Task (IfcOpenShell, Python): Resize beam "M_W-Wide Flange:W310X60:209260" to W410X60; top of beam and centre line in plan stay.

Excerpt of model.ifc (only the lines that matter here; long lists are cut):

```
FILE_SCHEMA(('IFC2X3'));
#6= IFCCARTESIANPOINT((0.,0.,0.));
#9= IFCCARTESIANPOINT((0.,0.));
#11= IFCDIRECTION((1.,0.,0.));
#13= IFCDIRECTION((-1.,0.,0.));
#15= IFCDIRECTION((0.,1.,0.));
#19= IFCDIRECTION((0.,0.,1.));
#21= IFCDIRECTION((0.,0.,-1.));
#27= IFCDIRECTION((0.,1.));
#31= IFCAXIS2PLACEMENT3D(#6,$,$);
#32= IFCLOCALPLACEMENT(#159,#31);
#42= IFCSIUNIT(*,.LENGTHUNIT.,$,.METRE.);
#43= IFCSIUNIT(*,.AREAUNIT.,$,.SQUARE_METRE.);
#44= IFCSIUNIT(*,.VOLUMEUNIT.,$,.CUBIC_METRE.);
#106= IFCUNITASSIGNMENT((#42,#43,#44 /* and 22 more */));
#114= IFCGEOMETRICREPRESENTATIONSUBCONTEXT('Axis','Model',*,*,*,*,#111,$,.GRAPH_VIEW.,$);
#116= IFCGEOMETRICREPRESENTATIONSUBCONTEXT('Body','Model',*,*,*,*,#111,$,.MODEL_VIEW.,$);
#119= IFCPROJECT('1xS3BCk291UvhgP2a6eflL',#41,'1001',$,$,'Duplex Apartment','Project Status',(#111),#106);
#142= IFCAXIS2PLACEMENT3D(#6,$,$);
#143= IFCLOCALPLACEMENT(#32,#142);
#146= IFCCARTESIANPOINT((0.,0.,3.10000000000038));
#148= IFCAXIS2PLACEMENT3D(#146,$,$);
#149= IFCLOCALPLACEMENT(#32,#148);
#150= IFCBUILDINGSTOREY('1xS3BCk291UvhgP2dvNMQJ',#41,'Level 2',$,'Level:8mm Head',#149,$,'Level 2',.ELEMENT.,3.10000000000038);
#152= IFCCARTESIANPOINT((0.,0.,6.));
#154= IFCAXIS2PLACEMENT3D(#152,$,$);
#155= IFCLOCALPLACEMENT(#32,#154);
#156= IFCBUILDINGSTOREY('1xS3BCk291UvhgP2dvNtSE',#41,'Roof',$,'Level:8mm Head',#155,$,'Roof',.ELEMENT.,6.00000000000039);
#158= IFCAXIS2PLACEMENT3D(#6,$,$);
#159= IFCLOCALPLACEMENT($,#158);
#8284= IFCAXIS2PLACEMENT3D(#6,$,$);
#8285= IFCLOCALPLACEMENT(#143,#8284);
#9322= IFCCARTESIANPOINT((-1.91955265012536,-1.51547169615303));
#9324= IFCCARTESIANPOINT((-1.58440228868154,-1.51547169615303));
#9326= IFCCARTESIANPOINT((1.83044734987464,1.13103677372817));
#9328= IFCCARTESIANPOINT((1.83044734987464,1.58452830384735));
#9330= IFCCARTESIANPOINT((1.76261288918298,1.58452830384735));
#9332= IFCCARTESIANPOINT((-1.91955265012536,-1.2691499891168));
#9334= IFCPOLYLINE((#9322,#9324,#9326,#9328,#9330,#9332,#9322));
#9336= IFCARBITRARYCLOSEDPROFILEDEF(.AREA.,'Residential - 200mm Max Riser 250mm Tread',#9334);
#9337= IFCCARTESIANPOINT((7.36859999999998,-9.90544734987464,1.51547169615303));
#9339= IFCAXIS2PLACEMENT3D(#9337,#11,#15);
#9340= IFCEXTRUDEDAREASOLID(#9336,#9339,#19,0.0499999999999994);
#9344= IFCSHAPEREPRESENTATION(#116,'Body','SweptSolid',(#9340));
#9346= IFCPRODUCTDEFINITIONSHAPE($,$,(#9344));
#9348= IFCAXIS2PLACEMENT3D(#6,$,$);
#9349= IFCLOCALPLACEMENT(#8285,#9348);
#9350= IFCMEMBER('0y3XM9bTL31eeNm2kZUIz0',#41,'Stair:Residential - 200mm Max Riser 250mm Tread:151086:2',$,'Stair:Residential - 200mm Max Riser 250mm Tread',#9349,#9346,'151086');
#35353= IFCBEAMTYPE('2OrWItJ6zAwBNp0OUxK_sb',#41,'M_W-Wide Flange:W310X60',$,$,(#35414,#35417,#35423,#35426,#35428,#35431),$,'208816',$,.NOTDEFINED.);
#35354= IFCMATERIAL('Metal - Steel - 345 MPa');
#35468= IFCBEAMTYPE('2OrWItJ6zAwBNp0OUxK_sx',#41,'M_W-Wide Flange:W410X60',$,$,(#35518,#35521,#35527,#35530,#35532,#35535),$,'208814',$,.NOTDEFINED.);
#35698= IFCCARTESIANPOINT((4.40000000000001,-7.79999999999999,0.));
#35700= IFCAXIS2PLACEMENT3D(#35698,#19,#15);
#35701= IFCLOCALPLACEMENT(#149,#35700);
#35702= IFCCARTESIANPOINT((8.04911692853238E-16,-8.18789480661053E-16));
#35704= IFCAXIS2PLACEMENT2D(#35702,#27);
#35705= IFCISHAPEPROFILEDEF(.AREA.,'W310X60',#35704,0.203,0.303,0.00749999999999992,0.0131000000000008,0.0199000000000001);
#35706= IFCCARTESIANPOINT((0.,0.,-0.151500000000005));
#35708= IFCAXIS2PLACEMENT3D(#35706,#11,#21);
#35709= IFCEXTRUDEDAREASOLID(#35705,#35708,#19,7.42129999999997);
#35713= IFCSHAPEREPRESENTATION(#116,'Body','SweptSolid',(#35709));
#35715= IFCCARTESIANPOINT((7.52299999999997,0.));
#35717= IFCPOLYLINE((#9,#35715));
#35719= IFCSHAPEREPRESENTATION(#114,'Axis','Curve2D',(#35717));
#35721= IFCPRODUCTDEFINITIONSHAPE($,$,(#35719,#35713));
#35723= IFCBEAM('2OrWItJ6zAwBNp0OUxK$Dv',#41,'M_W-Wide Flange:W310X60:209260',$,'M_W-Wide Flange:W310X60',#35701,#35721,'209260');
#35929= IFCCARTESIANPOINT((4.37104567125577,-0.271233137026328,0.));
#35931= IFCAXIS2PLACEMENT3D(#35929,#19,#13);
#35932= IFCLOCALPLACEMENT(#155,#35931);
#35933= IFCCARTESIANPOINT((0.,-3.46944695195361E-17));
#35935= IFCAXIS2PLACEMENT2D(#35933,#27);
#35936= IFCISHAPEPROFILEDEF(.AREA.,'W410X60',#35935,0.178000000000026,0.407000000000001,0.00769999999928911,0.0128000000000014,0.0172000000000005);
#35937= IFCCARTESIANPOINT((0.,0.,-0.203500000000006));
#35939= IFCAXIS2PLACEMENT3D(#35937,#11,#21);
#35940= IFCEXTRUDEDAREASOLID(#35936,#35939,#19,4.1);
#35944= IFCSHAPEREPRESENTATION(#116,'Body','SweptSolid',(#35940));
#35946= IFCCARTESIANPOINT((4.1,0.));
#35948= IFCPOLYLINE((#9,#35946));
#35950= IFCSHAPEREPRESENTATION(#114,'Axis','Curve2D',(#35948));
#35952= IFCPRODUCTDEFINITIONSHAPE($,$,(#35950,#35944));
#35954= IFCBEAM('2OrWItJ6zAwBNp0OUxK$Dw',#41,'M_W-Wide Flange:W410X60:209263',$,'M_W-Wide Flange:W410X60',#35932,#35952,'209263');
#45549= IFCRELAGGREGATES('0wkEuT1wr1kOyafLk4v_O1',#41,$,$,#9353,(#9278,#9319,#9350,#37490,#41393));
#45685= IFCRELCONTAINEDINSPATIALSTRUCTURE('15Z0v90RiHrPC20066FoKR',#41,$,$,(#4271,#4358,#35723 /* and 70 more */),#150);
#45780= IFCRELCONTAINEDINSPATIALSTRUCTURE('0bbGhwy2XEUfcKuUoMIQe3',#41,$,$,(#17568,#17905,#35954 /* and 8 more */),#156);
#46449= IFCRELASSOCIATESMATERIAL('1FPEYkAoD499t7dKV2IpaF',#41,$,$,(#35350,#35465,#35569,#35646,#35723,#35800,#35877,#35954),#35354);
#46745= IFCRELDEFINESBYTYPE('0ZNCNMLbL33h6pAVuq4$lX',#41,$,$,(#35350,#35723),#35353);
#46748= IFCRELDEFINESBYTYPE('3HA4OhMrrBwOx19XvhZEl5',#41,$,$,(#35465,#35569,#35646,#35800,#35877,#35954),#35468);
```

```python
import ifcopenshell
import ifcopenshell.api.type
import ifcopenshell.util.element
import ifcopenshell.util.representation

model = ifcopenshell.open("model.ifc")

member = model.by_id(35723)
source = next(p for p in model.by_type("IfcIShapeProfileDef") if p.ProfileName == "W410X60")

body = ifcopenshell.util.representation.get_representation(member, "Model", "Body")
solid = body.Items[0]
old_profile = solid.SweptArea

# Copy the section's sizes but keep this member's own profile position.
profile = ifcopenshell.util.element.copy(model, source)
# Profiles are centred, so shift by half the change in depth to hold the top.
shift = (old_profile.OverallDepth - profile.OverallDepth) / 2
x, y = old_profile.Position.Location.Coordinates
up = (-1.0, 0.0)  # upwards, in the solid's own plane
location = model.createIfcCartesianPoint((x + up[0] * shift, y + up[1] * shift))
profile.Position = model.createIfcAxis2Placement2D(location, old_profile.Position.RefDirection)
solid.SweptArea = profile
if not model.get_total_inverses(old_profile):
    ifcopenshell.util.element.remove_deep2(model, old_profile)

new_type = model.by_id(35468)
ifcopenshell.api.type.assign_type(
    model, related_objects=[member], relating_type=new_type, should_map_representations=False
)
member.Name = member.Name.replace("W310X60", "W410X60")
member.ObjectType = "M_W-Wide Flange:W410X60"

print(solid.SweptArea)

model.write("model_edited.ifc")
```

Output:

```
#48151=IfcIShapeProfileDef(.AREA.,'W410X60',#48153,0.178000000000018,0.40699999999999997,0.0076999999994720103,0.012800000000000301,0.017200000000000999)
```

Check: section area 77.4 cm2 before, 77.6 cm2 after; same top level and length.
